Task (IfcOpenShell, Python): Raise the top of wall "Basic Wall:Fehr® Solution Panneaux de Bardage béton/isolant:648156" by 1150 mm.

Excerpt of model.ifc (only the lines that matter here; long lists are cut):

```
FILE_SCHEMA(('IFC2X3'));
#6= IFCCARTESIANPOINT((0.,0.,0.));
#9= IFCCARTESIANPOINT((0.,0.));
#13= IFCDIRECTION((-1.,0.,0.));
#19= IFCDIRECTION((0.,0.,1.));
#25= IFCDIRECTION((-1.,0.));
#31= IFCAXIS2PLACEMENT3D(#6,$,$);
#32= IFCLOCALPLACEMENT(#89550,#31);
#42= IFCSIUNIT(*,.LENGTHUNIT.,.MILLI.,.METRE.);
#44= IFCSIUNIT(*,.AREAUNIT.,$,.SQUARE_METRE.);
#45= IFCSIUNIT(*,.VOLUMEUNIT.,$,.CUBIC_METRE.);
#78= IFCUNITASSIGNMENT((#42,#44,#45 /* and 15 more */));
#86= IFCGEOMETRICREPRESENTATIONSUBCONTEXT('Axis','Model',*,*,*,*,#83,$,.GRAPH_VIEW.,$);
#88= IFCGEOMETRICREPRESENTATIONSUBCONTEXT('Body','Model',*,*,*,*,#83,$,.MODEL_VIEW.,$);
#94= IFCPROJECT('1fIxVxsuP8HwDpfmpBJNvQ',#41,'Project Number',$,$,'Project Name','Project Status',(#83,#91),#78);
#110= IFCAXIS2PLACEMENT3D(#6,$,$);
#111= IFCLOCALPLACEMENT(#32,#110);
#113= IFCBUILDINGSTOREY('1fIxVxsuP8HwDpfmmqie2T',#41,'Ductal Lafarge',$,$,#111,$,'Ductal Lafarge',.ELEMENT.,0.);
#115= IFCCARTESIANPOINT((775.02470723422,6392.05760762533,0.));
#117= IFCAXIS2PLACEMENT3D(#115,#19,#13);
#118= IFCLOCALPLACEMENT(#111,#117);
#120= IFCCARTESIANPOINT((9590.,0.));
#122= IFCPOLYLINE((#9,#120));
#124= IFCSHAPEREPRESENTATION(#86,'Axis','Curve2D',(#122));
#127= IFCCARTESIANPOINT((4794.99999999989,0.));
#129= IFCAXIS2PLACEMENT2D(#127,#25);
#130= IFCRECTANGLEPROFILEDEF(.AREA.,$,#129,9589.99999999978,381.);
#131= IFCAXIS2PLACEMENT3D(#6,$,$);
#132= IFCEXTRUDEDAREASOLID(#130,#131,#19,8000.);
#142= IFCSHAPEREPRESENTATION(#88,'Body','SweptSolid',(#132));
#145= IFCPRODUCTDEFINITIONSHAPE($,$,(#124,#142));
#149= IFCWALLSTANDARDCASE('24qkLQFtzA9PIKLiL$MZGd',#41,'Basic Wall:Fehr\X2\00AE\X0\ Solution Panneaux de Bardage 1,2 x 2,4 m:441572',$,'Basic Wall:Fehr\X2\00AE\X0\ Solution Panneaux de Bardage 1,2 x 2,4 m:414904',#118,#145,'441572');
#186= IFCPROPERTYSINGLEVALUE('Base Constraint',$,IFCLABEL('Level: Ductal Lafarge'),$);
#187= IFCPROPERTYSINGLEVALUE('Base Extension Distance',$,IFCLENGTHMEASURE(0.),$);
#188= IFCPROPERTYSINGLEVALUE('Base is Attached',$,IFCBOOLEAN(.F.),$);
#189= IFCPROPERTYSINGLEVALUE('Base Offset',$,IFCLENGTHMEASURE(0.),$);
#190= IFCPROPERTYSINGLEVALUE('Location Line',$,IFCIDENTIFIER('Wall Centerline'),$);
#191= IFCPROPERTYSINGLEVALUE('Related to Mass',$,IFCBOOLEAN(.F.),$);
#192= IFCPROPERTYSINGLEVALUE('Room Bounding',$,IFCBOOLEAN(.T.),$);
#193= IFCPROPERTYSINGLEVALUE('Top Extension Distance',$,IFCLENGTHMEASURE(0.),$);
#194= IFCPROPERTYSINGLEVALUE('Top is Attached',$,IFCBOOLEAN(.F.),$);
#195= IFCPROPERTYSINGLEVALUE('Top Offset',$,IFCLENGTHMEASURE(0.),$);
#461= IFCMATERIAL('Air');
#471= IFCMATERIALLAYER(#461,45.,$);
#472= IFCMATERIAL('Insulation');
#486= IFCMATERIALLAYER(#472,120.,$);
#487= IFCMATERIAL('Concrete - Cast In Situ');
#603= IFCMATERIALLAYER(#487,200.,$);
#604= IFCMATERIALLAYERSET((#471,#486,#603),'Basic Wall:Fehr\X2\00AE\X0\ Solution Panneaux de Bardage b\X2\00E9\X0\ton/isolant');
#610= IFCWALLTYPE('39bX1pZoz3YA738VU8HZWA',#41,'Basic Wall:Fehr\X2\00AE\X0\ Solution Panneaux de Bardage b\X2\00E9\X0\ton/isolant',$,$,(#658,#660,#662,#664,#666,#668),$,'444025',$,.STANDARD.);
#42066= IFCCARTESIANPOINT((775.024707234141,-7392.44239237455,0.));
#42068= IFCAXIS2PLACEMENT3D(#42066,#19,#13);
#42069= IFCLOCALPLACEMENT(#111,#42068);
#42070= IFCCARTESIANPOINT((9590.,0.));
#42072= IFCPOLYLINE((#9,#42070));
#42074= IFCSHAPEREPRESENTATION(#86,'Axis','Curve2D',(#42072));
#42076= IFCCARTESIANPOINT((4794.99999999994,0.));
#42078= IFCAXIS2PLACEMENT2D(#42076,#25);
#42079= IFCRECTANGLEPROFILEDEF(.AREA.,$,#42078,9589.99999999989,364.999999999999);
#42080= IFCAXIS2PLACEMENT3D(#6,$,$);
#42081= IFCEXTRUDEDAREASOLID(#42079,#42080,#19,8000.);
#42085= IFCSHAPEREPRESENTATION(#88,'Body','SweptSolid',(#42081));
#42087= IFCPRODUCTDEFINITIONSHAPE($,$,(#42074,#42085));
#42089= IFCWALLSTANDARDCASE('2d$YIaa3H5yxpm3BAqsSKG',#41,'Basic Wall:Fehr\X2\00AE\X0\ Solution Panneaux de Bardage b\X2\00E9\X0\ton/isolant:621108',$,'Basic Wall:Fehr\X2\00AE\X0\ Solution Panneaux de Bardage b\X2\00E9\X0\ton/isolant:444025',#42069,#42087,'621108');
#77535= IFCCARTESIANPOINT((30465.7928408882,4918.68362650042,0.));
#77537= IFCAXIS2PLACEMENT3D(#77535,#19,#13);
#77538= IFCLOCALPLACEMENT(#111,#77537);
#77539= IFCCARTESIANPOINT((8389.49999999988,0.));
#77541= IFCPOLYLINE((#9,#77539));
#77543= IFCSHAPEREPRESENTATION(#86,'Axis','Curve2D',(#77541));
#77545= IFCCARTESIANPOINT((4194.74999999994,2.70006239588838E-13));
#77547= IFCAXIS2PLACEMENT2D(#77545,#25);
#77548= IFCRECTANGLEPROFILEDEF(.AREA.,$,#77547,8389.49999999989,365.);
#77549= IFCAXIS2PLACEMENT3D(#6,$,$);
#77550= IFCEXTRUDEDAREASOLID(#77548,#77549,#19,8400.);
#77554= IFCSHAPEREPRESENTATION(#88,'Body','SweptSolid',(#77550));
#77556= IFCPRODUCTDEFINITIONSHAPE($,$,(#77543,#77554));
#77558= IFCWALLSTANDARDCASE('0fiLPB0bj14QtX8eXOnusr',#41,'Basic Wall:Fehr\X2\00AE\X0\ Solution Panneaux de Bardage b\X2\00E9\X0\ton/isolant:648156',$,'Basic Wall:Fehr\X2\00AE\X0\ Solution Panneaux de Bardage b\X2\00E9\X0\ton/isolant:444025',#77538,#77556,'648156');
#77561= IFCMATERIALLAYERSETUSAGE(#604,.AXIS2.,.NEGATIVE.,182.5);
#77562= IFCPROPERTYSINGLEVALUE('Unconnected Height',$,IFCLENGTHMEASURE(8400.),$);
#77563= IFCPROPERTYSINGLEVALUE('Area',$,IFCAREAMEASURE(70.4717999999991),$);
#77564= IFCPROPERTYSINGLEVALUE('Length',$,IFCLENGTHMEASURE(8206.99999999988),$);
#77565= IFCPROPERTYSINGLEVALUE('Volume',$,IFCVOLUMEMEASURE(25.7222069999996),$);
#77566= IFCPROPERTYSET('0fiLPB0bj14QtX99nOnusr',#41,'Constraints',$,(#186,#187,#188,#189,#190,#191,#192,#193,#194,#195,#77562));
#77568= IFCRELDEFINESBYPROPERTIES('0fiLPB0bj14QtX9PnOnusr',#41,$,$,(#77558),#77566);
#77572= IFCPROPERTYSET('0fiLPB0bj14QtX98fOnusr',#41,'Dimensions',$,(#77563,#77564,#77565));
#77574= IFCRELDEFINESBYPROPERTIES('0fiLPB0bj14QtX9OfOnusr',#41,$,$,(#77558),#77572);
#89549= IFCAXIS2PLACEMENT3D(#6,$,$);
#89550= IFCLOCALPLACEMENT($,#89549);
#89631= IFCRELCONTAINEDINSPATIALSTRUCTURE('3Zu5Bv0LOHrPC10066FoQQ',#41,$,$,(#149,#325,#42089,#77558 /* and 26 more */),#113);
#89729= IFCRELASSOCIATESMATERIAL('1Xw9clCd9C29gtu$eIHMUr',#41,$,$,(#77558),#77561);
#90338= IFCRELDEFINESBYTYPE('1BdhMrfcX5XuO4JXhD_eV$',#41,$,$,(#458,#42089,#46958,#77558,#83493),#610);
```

```python
import ifcopenshell
import ifcopenshell.api.pset
import ifcopenshell.geom
import ifcopenshell.util.element
import ifcopenshell.util.representation
import ifcopenshell.util.shape
import ifcopenshell.util.unit

model = ifcopenshell.open("model.ifc")
unit_scale = ifcopenshell.util.unit.calculate_unit_scale(model)
area_scale = ifcopenshell.util.unit.calculate_unit_scale(model, "AREAUNIT")
volume_scale = ifcopenshell.util.unit.calculate_unit_scale(model, "VOLUMEUNIT")
settings = ifcopenshell.geom.settings()


def volume(element):
    """Net volume in cubic metres, openings subtracted."""
    shape = ifcopenshell.geom.create_shape(settings, element)
    return ifcopenshell.util.shape.get_volume(shape.geometry)


wall = model.by_guid("0fiLPB0bj14QtX8eXOnusr")
before = volume(wall)

body = ifcopenshell.util.representation.get_representation(wall, "Model", "Body")
solid = body.Items[0]
old_height = solid.Depth
solid.Depth += 1.15 / unit_scale
after = volume(wall)
thickness = 0.365  # wall thickness in metres

# Update the stored height, areas and volumes.
pset = model.by_id(ifcopenshell.util.element.get_pset(wall, "Constraints", should_inherit=False)["id"])
ifcopenshell.api.pset.edit_pset(model, pset=pset, properties={
    "Unconnected Height": model.create_entity("IfcLengthMeasure", solid.Depth),
})
pset = model.by_id(ifcopenshell.util.element.get_pset(wall, "Dimensions", should_inherit=False)["id"])
ifcopenshell.api.pset.edit_pset(model, pset=pset, properties={
    "Area": model.create_entity("IfcAreaMeasure", after / thickness / area_scale),
    "Volume": model.create_entity("IfcVolumeMeasure", after / volume_scale),
})

print(f"height {old_height:g} -> {solid.Depth:g}, volume {before:.3f} -> {after:.3f} m3")

model.write("model_updated.ifc")
```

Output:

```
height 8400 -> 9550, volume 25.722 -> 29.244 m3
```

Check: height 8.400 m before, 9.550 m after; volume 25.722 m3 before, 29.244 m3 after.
